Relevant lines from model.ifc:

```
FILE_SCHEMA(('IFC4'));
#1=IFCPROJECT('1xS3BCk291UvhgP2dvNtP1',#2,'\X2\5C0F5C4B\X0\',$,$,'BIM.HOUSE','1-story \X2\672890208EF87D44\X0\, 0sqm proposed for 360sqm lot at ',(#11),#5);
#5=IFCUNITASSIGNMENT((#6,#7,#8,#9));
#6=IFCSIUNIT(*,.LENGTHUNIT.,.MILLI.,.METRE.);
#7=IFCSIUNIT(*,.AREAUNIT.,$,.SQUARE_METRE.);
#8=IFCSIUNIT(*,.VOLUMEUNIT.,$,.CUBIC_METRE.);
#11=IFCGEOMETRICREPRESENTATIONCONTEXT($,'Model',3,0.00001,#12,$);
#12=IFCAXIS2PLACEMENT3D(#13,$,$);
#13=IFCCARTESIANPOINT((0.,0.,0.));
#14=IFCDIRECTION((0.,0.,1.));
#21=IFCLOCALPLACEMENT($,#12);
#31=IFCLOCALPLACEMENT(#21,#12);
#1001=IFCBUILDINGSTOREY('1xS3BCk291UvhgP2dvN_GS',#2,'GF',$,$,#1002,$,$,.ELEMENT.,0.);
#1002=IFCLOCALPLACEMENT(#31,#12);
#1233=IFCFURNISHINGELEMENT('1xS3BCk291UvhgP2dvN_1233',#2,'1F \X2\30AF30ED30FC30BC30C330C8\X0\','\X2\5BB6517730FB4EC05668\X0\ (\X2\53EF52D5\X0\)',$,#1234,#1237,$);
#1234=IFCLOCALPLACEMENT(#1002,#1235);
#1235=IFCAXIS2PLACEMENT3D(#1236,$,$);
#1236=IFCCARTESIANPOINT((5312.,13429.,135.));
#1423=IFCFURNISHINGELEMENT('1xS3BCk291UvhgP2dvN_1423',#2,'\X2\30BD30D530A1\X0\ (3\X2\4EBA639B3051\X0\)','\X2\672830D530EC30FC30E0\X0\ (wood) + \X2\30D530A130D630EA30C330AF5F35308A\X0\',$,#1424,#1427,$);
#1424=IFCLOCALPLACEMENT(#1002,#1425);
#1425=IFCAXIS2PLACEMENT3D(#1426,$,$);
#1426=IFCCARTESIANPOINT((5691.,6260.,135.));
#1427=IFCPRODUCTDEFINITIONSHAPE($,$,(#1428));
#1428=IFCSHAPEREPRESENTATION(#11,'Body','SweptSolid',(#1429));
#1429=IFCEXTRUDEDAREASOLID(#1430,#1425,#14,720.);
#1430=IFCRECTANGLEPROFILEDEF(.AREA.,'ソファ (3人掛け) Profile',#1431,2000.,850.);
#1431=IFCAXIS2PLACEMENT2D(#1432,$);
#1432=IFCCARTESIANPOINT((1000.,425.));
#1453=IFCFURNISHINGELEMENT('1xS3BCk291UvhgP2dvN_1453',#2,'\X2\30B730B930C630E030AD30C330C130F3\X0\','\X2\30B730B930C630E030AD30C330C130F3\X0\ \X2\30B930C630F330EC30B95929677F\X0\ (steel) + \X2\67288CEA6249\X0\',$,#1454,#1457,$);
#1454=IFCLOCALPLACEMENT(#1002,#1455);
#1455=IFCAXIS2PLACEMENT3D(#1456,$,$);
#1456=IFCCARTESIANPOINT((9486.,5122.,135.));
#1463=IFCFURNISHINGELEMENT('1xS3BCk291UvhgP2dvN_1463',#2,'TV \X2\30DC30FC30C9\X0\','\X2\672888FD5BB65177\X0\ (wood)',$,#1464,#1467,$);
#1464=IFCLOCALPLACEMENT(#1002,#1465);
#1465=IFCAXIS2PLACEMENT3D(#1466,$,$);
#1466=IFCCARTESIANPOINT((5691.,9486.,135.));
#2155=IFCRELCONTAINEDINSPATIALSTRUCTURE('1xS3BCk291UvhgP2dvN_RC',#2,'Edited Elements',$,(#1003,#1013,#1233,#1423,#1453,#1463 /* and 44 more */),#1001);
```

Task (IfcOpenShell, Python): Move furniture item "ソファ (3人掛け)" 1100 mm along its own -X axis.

```python
import ifcopenshell
import ifcopenshell.api.geometry
import ifcopenshell.util.placement
import ifcopenshell.util.unit

model = ifcopenshell.open("model.ifc")
unit_scale = ifcopenshell.util.unit.calculate_unit_scale(model)

item = model.by_guid("1xS3BCk291UvhgP2dvN_1423")
matrix = ifcopenshell.util.placement.get_local_placement(item.ObjectPlacement)
matrix[:3, 3] -= matrix[:3, 0] * 1.1 / unit_scale
ifcopenshell.api.geometry.edit_object_placement(model, product=item, matrix=matrix, is_si=False)

print(ifcopenshell.util.placement.get_local_placement(item.ObjectPlacement).round(3) + 0.0)

model.write("model_updated.ifc")
```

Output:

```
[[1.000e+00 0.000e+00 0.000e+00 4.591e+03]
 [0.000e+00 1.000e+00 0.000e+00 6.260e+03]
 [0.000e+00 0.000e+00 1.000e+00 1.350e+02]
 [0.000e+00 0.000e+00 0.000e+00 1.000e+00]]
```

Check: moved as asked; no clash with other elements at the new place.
